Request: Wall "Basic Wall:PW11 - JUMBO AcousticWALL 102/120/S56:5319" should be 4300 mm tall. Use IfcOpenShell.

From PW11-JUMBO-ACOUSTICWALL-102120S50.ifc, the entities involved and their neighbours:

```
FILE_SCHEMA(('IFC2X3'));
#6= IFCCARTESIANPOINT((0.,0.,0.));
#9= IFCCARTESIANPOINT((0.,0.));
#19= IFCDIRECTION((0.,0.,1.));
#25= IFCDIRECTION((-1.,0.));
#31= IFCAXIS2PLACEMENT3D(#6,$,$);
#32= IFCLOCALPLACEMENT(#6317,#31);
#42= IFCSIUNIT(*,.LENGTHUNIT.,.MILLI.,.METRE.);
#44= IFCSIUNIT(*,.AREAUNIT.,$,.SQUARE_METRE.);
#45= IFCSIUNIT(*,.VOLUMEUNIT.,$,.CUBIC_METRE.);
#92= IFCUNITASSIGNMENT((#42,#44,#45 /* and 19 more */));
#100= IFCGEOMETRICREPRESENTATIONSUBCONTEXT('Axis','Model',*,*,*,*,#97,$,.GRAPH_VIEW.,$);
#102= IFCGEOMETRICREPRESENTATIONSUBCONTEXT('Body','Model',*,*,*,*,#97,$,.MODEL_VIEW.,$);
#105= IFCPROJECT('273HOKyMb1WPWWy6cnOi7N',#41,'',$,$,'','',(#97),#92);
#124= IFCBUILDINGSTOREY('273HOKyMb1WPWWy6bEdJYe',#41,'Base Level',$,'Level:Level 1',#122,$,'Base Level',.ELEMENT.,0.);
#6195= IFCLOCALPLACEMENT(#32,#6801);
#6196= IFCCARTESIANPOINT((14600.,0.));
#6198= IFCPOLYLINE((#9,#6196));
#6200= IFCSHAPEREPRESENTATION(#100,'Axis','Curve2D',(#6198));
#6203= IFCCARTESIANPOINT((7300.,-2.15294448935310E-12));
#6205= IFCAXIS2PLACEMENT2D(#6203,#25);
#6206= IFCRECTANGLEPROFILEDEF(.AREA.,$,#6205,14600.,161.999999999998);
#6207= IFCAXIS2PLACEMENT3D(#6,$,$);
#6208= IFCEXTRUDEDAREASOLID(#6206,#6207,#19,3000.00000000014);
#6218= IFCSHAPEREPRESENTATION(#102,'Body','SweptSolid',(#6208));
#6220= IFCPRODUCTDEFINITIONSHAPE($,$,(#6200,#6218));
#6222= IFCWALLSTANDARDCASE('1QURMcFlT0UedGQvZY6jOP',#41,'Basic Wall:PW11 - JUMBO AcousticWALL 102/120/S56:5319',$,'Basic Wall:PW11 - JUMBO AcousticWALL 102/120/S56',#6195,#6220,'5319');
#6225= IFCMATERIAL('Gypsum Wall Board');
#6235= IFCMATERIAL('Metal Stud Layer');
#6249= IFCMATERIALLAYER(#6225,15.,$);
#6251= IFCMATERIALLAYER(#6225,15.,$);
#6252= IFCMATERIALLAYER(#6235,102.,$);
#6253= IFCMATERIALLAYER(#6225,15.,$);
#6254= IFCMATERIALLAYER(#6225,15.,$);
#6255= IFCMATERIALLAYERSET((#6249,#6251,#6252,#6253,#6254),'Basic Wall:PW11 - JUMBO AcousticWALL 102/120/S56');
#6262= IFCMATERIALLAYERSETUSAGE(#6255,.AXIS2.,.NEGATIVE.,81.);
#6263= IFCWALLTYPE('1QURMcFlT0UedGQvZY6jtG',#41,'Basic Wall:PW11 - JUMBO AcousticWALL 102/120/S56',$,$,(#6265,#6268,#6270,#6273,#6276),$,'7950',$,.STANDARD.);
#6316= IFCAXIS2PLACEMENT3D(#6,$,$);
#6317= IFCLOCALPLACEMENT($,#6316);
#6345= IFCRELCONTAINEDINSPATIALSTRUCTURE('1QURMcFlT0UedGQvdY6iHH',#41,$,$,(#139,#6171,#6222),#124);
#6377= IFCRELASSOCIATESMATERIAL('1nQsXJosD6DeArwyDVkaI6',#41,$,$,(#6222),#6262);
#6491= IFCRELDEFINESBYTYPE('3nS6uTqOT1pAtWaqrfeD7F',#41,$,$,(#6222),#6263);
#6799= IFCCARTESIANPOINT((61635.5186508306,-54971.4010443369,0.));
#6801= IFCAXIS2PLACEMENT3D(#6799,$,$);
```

```python
import ifcopenshell
import ifcopenshell.geom
import ifcopenshell.util.representation
import ifcopenshell.util.shape
import ifcopenshell.util.unit

model = ifcopenshell.open("PW11-JUMBO-ACOUSTICWALL-102120S50.ifc")
unit_scale = ifcopenshell.util.unit.calculate_unit_scale(model)
settings = ifcopenshell.geom.settings()


def volume(element):
    """Net volume in cubic metres, openings subtracted."""
    shape = ifcopenshell.geom.create_shape(settings, element)
    return ifcopenshell.util.shape.get_volume(shape.geometry)


wall = model.by_guid("1QURMcFlT0UedGQvZY6jOP")
before = volume(wall)

body = ifcopenshell.util.representation.get_representation(wall, "Model", "Body")
solid = body.Items[0]
old_height = solid.Depth
solid.Depth = 4.3 / unit_scale
after = volume(wall)

print(f"height {old_height:g} -> {solid.Depth:g}, volume {before:.3f} -> {after:.3f} m3")

model.write("PW11-JUMBO-ACOUSTICWALL-102120S50_v2.ifc")
```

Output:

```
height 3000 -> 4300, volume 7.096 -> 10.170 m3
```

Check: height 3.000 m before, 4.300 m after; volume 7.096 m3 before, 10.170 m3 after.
